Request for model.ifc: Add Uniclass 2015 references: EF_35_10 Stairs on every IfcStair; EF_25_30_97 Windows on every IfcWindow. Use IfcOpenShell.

First a look at what the model holds.

```python
import ifcopenshell

model = ifcopenshell.open("model.ifc")
print(model.schema)
print("classifications:", [c.Name for c in model.by_type("IfcClassification")])
for ifc_class in ("IfcDoor", "IfcRoof", "IfcStair", "IfcWall", "IfcWindow"):
    print(ifc_class, len(model.by_type(ifc_class)))
```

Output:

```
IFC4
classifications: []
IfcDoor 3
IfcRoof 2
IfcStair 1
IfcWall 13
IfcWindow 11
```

```python
import ifcopenshell
import ifcopenshell.api.classification

model = ifcopenshell.open("model.ifc")

system = ifcopenshell.api.classification.add_classification(model, classification="Uniclass 2015")

codes = {
    "IfcStair": ("EF_35_10", "Stairs"),
    "IfcWindow": ("EF_25_30_97", "Windows"),
}
for ifc_class, (code, name) in codes.items():
    products = model.by_type(ifc_class)
    ifcopenshell.api.classification.add_reference(
        model, products=products, classification=system, identification=code, name=name
    )
    print(code, len(products))

model.write("model-out.ifc")
```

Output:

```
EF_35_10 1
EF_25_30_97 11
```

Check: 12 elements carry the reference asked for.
